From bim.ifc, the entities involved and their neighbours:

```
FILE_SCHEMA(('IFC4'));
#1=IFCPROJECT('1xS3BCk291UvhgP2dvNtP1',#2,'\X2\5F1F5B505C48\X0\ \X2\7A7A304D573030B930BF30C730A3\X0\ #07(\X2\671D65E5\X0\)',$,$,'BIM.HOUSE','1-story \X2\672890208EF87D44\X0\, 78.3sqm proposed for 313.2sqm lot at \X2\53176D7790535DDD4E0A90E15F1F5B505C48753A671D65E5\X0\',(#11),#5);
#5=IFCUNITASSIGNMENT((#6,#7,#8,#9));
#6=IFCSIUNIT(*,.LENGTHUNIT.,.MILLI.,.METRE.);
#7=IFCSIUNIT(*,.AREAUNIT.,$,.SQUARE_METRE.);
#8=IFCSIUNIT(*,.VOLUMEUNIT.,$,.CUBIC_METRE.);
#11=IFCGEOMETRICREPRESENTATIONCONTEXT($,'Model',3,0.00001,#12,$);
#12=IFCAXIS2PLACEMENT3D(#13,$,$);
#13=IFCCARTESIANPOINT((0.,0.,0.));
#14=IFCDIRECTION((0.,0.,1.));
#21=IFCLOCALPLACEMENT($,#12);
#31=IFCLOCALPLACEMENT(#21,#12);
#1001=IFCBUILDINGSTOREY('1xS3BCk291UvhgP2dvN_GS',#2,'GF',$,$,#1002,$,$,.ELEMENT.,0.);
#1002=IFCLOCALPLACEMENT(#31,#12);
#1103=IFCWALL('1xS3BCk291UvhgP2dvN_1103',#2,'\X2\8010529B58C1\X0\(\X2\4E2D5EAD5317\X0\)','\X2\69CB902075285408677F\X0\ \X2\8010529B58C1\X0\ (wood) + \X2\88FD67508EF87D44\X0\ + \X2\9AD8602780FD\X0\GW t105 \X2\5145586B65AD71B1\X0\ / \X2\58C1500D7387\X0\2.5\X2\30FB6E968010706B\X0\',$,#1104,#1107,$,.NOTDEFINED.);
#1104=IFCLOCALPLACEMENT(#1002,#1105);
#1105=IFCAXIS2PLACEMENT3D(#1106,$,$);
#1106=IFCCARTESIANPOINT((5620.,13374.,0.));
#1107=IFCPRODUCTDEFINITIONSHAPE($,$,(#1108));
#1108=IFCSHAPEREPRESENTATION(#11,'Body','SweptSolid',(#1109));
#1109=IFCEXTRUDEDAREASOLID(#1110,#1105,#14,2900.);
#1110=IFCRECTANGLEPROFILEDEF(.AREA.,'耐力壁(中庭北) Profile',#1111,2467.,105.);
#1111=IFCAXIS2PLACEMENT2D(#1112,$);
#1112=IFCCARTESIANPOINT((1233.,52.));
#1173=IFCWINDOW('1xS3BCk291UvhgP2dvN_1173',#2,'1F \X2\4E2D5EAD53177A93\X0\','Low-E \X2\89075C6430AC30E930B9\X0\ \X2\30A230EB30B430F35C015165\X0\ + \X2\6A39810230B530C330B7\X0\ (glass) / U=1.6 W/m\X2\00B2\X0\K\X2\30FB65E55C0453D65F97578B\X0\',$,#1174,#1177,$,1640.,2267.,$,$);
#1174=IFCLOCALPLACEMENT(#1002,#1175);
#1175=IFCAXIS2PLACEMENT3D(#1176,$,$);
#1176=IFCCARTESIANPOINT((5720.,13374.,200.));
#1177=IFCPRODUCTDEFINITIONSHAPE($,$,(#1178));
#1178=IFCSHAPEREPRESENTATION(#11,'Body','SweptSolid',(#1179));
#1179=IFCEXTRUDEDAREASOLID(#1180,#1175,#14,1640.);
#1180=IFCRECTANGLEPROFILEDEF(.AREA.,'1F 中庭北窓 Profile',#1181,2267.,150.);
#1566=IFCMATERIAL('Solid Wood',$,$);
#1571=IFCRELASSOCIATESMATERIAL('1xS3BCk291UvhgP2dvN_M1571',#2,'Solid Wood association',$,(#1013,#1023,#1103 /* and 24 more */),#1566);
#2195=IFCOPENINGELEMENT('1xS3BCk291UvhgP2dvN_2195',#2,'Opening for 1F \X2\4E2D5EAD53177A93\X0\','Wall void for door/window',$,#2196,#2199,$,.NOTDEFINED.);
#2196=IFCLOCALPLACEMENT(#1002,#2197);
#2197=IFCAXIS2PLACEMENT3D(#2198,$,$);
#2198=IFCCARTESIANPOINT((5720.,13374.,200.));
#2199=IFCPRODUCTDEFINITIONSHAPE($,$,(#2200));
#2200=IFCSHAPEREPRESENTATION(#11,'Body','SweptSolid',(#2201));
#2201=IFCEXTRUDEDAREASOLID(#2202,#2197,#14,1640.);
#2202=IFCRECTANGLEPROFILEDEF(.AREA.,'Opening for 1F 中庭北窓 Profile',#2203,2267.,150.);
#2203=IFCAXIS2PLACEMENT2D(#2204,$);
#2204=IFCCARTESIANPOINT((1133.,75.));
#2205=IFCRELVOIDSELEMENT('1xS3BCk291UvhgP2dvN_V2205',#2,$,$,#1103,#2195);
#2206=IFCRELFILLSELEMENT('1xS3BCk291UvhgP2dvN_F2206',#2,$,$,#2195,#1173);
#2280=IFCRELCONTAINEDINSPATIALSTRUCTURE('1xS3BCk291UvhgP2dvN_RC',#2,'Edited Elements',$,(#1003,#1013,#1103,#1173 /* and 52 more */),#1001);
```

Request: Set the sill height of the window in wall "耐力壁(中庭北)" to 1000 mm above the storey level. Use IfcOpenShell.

```python
import numpy as np
import ifcopenshell
import ifcopenshell.api.geometry
import ifcopenshell.geom
import ifcopenshell.util.element
import ifcopenshell.util.placement
import ifcopenshell.util.shape
import ifcopenshell.util.unit

model = ifcopenshell.open("bim.ifc")
unit_scale = ifcopenshell.util.unit.calculate_unit_scale(model)

window = model.by_guid("1xS3BCk291UvhgP2dvN_1173")
opening = window.FillsVoids[0].RelatingOpeningElement
storey = ifcopenshell.util.element.get_container(window, ifc_class="IfcBuildingStorey")
level = ifcopenshell.util.placement.get_local_placement(storey.ObjectPlacement)[2, 3]

# The opening's origin need not be at the sill, so measure its lowest point.
shape = ifcopenshell.geom.create_shape(ifcopenshell.geom.settings(), opening)
bottom = ifcopenshell.util.shape.get_shape_bottom_elevation(shape, shape.geometry) / unit_scale
dz = level + 1 / unit_scale - bottom

shift = np.array([0.0, 0.0, dz])
# The window is not placed relative to its opening, so move both.
for product in (opening, window):
    matrix = ifcopenshell.util.placement.get_local_placement(product.ObjectPlacement)
    matrix[:3, 3] += shift
    ifcopenshell.api.geometry.edit_object_placement(model, product=product, matrix=matrix, is_si=False)

print(f"moved by {dz * unit_scale:+.3f} m")

model.write("bim_edited.ifc")
```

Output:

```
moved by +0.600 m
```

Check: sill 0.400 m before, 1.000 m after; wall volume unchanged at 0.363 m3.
